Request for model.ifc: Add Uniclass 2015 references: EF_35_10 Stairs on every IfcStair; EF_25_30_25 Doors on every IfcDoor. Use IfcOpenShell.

First a look at what the model holds.

```python
import ifcopenshell

model = ifcopenshell.open("model.ifc")
print(model.schema)
print("classifications:", [c.Name for c in model.by_type("IfcClassification")])
for ifc_class in ("IfcDoor", "IfcRoof", "IfcStair", "IfcWall", "IfcWindow"):
    print(ifc_class, len(model.by_type(ifc_class)))
```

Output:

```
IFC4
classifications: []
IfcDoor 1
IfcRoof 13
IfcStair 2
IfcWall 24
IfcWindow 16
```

```python
import ifcopenshell
import ifcopenshell.api.classification

model = ifcopenshell.open("model.ifc")

system = ifcopenshell.api.classification.add_classification(model, classification="Uniclass 2015")

codes = {
    "IfcStair": ("EF_35_10", "Stairs"),
    "IfcDoor": ("EF_25_30_25", "Doors"),
}
for ifc_class, (code, name) in codes.items():
    products = model.by_type(ifc_class)
    ifcopenshell.api.classification.add_reference(
        model, products=products, classification=system, identification=code, name=name
    )
    print(code, len(products))

model.write("model_v2.ifc")
```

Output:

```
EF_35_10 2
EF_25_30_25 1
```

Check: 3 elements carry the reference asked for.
